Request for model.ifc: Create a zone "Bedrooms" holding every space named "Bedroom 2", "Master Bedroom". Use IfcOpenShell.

First a look at what the model holds.

```python
import ifcopenshell

model = ifcopenshell.open("model.ifc")
print(model.schema)
seen = {}
for space in model.by_type("IfcSpace"):
    seen[space.LongName] = seen.get(space.LongName, 0) + 1
for name, count in sorted(seen.items(), key=str):
    print(count, "x", name)
print("zones:", [z.Name for z in model.by_type("IfcZone")][:20])
```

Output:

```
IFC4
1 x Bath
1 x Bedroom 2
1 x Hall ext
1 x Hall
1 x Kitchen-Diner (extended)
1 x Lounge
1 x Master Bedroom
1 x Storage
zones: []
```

```python
import ifcopenshell
import ifcopenshell.api.group
import ifcopenshell.api.root

model = ifcopenshell.open("model.ifc")

names = {"Bedroom 2", "Master Bedroom"}
spaces = [s for s in model.by_type("IfcSpace") if s.LongName in names]

zone = ifcopenshell.api.root.create_entity(model, ifc_class="IfcZone", name="Bedrooms")
ifcopenshell.api.group.assign_group(model, products=spaces, group=zone)
print(len(spaces), "spaces in", zone.Name)

model.write("model_edited.ifc")
```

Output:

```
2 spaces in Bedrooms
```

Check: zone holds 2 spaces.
